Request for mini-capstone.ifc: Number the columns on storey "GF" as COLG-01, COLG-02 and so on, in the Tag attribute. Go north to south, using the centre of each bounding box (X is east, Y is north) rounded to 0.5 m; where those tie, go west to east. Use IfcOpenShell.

First a look at what the model holds.

```python
import ifcopenshell
import ifcopenshell.util.element
import ifcopenshell.util.placement

model = ifcopenshell.open("mini-capstone.ifc")
print(model.schema)
storey = next(s for s in model.by_type("IfcBuildingStorey") if s.Name == "GF")
columns = [e for e in ifcopenshell.util.element.get_decomposition(storey) if e.is_a("IfcColumn")]
for e in sorted(columns, key=lambda e: e.id()):
    origin = ifcopenshell.util.placement.get_local_placement(e.ObjectPlacement)[:3, 3]
    print(e.id(), e.Tag, e.Name, origin.round(2) + 0.0, sep=" | ")
```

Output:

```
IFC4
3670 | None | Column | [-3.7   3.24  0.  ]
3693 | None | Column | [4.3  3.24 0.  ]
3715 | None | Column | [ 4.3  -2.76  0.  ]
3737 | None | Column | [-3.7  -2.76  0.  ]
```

```python
import ifcopenshell
import ifcopenshell.geom
import ifcopenshell.util.element
import ifcopenshell.util.shape

model = ifcopenshell.open("mini-capstone.ifc")
settings = ifcopenshell.geom.settings()
settings.set("use-world-coords", True)


def centre(element):
    shape = ifcopenshell.geom.create_shape(settings, element)
    return ifcopenshell.util.shape.get_bbox_centroid(shape.geometry)


storey = next(s for s in model.by_type("IfcBuildingStorey") if s.Name == "GF")
columns = [e for e in ifcopenshell.util.element.get_decomposition(storey) if e.is_a("IfcColumn")]

# Insertion points can sit at a corner or the storey origin, so sort by the geometry (in metres).
centres = {e: centre(e) for e in columns}
columns.sort(key=lambda e: (-round(centres[e][1] / 0.5), centres[e][0]))

for i, e in enumerate(columns, start=1):
    number = f"COLG-{i:02d}"
    e.Tag = number
    print(e.id(), number)

model.write("mini-capstone_rev.ifc")
```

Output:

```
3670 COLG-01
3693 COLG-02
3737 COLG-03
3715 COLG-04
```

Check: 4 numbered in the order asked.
